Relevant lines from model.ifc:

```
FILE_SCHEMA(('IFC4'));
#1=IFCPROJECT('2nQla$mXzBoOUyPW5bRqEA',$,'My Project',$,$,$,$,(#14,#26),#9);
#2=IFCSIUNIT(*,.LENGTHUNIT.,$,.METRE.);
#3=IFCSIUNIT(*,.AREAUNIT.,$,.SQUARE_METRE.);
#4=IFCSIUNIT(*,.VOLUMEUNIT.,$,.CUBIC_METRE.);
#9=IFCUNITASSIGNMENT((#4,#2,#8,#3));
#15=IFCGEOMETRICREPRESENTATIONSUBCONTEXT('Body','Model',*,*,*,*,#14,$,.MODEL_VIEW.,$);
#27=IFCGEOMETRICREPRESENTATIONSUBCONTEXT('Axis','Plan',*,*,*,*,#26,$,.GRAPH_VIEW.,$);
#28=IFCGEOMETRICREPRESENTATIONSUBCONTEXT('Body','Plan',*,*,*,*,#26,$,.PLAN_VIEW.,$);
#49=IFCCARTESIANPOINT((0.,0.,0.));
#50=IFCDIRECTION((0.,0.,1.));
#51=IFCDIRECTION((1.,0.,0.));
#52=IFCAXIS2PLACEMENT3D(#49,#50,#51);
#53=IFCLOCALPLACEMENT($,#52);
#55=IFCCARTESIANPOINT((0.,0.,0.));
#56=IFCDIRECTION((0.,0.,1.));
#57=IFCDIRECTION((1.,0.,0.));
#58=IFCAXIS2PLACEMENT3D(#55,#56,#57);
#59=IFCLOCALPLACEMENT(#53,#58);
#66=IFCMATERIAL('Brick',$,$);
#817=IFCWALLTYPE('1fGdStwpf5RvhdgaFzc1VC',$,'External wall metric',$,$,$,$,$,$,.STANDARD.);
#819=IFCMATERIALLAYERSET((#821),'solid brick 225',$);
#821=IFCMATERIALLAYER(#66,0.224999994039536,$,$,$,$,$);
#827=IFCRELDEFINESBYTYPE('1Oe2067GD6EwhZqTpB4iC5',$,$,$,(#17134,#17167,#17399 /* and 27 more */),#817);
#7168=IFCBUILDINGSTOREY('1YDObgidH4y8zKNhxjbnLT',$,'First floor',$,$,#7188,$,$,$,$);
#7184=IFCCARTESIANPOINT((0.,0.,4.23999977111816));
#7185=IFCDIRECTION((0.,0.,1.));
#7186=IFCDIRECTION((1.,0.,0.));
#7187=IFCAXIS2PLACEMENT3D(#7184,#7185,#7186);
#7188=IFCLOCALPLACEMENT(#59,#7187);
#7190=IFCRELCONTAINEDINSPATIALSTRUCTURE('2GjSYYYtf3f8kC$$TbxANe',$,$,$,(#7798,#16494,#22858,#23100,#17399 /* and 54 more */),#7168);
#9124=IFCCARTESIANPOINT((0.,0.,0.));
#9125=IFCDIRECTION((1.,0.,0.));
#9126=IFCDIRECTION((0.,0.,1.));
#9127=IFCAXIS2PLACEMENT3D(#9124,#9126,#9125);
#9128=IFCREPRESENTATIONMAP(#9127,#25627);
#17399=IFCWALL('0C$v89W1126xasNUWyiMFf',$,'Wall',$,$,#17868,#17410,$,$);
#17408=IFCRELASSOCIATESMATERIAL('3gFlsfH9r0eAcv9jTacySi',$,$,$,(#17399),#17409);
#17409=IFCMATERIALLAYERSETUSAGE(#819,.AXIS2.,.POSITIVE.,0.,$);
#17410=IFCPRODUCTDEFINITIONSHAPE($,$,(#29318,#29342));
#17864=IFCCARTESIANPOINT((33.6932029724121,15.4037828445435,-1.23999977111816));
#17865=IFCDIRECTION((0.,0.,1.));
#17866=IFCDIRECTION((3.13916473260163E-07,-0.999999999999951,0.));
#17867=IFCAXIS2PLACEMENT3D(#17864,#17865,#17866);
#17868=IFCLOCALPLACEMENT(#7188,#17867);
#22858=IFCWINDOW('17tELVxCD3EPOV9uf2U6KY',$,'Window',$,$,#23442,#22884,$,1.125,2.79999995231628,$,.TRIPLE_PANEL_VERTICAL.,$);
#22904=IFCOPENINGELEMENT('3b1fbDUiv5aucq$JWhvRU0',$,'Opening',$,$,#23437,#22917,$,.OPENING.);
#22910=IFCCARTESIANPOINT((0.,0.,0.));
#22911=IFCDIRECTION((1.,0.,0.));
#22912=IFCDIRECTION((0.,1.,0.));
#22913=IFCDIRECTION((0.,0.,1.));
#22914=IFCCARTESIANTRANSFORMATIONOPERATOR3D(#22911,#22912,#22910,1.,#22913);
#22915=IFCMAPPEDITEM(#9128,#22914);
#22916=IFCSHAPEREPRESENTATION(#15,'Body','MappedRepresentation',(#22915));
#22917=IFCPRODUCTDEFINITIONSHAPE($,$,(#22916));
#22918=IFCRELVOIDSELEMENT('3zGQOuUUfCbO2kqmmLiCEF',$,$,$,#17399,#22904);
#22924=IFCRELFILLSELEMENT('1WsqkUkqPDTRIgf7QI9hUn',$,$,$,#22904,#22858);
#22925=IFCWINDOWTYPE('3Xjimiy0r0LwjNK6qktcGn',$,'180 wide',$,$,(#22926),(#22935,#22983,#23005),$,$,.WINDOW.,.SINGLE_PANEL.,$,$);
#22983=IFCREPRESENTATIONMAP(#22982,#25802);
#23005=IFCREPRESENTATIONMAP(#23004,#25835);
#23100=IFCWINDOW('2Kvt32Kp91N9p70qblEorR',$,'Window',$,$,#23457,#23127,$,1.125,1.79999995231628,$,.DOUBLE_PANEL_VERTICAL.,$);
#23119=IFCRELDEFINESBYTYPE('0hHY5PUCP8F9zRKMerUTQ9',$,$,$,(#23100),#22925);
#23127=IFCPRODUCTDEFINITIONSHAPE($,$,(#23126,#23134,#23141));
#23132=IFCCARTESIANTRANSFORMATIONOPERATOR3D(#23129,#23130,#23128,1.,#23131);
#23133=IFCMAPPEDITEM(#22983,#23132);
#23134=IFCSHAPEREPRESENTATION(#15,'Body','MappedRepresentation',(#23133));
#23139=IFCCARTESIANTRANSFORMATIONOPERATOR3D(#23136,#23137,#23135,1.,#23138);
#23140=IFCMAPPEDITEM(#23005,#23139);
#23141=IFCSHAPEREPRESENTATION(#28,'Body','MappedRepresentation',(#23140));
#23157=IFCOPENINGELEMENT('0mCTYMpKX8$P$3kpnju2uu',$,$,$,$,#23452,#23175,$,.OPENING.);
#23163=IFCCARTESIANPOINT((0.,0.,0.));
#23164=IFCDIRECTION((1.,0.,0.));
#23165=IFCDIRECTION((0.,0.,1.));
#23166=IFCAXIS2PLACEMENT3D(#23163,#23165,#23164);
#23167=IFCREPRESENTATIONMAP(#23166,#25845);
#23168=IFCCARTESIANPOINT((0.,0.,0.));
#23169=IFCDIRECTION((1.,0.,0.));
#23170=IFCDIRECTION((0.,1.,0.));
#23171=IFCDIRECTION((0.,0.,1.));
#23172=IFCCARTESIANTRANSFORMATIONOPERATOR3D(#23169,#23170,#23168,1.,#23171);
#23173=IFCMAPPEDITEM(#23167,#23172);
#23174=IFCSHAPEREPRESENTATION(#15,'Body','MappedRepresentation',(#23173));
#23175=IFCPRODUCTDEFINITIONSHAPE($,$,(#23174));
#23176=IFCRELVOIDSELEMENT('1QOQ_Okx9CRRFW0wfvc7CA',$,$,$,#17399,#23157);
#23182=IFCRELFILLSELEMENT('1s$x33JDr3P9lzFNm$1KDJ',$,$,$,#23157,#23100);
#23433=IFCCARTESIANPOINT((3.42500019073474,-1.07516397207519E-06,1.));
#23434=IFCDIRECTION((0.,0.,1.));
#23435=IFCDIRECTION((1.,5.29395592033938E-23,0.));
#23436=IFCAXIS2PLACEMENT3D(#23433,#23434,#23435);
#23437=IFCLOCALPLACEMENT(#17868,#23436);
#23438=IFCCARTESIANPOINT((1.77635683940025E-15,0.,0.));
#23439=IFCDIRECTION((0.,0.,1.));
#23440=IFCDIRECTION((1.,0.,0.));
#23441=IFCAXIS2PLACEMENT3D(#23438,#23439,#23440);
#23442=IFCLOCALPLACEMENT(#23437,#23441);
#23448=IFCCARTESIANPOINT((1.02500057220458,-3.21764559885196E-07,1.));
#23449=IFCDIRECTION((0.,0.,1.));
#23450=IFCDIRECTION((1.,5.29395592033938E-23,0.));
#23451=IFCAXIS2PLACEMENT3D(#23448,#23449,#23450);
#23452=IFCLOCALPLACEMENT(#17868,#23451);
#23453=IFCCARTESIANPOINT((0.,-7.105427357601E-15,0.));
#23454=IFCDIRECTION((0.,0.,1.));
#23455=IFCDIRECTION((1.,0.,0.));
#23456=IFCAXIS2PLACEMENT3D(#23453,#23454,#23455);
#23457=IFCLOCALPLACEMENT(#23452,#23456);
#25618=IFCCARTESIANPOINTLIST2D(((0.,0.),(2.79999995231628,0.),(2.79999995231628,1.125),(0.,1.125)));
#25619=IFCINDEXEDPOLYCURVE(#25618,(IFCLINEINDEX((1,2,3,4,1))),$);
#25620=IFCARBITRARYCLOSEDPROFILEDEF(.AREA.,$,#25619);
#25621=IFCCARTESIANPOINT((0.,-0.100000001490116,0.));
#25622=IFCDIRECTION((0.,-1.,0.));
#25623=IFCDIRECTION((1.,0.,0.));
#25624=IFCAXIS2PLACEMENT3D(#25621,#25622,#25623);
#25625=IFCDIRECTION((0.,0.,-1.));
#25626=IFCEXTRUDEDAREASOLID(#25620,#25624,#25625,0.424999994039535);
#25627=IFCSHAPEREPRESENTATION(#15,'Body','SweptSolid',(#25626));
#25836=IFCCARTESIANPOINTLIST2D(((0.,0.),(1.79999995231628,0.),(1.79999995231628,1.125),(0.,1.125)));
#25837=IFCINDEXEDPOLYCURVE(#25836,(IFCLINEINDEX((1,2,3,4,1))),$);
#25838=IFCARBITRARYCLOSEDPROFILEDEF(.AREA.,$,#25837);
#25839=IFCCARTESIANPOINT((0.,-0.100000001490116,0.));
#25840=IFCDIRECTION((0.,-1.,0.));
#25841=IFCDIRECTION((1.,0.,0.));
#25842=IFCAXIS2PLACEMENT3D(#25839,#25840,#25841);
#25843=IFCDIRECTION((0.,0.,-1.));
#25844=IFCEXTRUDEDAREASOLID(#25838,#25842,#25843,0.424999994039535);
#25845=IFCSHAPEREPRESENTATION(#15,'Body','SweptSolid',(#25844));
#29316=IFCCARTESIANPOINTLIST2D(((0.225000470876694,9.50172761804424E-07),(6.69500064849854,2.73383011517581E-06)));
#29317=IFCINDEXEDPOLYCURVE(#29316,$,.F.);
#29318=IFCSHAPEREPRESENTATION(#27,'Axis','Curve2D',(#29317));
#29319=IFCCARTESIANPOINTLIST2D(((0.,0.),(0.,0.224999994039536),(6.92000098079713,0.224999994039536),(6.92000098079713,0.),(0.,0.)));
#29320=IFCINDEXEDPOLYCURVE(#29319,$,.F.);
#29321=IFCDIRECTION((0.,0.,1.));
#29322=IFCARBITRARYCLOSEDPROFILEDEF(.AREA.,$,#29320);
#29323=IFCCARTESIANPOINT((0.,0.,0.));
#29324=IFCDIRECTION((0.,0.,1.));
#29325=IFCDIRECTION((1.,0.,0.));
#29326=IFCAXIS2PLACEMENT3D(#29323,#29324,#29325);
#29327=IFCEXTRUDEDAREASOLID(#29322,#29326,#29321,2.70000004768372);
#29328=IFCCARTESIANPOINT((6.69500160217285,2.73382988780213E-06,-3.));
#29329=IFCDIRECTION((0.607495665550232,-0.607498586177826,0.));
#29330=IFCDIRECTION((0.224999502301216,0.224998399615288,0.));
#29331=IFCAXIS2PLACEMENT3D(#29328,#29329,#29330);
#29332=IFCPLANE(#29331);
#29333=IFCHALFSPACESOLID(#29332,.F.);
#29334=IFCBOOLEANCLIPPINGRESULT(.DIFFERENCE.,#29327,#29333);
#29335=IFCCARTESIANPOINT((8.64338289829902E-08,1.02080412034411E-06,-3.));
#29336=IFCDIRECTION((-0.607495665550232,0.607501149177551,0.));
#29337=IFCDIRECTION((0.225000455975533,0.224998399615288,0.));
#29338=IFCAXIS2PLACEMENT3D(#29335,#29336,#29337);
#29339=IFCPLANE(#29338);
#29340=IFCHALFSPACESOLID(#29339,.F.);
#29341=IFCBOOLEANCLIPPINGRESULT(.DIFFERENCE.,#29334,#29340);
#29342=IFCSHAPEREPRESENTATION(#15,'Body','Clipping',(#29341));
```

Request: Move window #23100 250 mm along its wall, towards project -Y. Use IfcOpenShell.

```python
import ifcopenshell
import ifcopenshell.api.geometry
import ifcopenshell.util.placement
import ifcopenshell.util.unit

model = ifcopenshell.open("model.ifc")
unit_scale = ifcopenshell.util.unit.calculate_unit_scale(model)

window = model.by_id(23100)
opening = window.FillsVoids[0].RelatingOpeningElement
wall = opening.VoidsElements[0].RelatingBuildingElement

wall_matrix = ifcopenshell.util.placement.get_local_placement(wall.ObjectPlacement)
shift = wall_matrix[:3, 0] * 0.25 / unit_scale
before = ifcopenshell.util.placement.get_local_placement(window.ObjectPlacement)[:3, 3].copy()

# The window is placed relative to its opening, so it follows when the opening moves.
matrix = ifcopenshell.util.placement.get_local_placement(opening.ObjectPlacement)
matrix[:3, 3] += shift
ifcopenshell.api.geometry.edit_object_placement(
    model, product=opening, matrix=matrix, is_si=False, should_transform_children=True
)

after = ifcopenshell.util.placement.get_local_placement(window.ObjectPlacement)[:3, 3]
print("window moved by", (after - before).round(3) + 0.0)

model.write("model_edited.ifc")
```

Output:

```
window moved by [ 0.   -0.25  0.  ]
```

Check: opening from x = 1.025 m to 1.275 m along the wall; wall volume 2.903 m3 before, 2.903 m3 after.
